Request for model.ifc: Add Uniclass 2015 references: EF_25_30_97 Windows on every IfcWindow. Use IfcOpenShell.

First a look at what the model holds.

```python
import ifcopenshell

model = ifcopenshell.open("model.ifc")
print(model.schema)
print("classifications:", [c.Name for c in model.by_type("IfcClassification")])
for ifc_class in ("IfcDoor", "IfcRoof", "IfcStair", "IfcWall", "IfcWindow"):
    print(ifc_class, len(model.by_type(ifc_class)))
```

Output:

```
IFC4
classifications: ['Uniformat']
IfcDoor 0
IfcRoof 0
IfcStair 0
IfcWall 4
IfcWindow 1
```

```python
import ifcopenshell
import ifcopenshell.api.classification

model = ifcopenshell.open("model.ifc")

system = ifcopenshell.api.classification.add_classification(model, classification="Uniclass 2015")

codes = {
    "IfcWindow": ("EF_25_30_97", "Windows"),
}
for ifc_class, (code, name) in codes.items():
    products = model.by_type(ifc_class)
    ifcopenshell.api.classification.add_reference(
        model, products=products, classification=system, identification=code, name=name
    )
    print(code, len(products))

model.write("model_rev.ifc")
```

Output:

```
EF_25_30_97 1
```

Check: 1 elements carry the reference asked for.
